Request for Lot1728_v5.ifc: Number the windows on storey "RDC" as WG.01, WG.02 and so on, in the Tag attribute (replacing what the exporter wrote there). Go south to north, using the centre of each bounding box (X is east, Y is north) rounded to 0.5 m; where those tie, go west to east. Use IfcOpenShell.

First a look at what the model holds.

```python
import ifcopenshell
import ifcopenshell.util.element
import ifcopenshell.util.placement

model = ifcopenshell.open("Lot1728_v5.ifc")
print(model.schema)
storey = next(s for s in model.by_type("IfcBuildingStorey") if s.Name == "RDC")
windows = [e for e in ifcopenshell.util.element.get_decomposition(storey) if e.is_a("IfcWindow")]
for e in sorted(windows, key=lambda e: e.id()):
    origin = ifcopenshell.util.placement.get_local_placement(e.ObjectPlacement)[:3, 3]
    print(e.id(), e.Tag, e.Name, origin.round(2) + 0.0, sep=" | ")
```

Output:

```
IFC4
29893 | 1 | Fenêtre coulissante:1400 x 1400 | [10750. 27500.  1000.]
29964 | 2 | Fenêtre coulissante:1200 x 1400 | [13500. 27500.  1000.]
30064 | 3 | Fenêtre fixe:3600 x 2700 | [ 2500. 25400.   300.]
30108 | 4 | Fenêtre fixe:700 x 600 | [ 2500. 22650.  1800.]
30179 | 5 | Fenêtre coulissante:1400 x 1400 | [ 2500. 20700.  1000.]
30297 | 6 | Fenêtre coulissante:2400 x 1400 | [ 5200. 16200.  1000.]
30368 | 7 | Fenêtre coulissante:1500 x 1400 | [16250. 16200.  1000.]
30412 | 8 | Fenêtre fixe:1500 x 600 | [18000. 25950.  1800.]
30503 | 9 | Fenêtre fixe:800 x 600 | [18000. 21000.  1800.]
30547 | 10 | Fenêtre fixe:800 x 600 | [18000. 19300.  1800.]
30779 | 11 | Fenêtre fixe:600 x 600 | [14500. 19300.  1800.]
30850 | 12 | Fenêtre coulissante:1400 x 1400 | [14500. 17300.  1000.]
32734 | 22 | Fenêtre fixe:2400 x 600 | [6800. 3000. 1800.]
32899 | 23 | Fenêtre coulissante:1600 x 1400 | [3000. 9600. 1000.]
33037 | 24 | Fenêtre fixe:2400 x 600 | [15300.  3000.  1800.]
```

```python
import ifcopenshell
import ifcopenshell.geom
import ifcopenshell.util.element
import ifcopenshell.util.shape

model = ifcopenshell.open("Lot1728_v5.ifc")
settings = ifcopenshell.geom.settings()
settings.set("use-world-coords", True)


def centre(element):
    shape = ifcopenshell.geom.create_shape(settings, element)
    return ifcopenshell.util.shape.get_bbox_centroid(shape.geometry)


storey = next(s for s in model.by_type("IfcBuildingStorey") if s.Name == "RDC")
windows = [e for e in ifcopenshell.util.element.get_decomposition(storey) if e.is_a("IfcWindow")]

# Insertion points can sit at a corner or the storey origin, so sort by the geometry (in metres).
centres = {e: centre(e) for e in windows}
windows.sort(key=lambda e: (round(centres[e][1] / 0.5), centres[e][0]))

for i, e in enumerate(windows, start=1):
    number = f"WG.{i:02d}"
    e.Tag = number
    print(e.id(), number)

model.write("Lot1728_v5-out.ifc")
```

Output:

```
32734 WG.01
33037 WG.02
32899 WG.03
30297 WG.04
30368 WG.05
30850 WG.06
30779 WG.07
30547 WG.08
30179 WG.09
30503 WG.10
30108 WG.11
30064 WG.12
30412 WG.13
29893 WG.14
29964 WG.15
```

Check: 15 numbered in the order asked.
